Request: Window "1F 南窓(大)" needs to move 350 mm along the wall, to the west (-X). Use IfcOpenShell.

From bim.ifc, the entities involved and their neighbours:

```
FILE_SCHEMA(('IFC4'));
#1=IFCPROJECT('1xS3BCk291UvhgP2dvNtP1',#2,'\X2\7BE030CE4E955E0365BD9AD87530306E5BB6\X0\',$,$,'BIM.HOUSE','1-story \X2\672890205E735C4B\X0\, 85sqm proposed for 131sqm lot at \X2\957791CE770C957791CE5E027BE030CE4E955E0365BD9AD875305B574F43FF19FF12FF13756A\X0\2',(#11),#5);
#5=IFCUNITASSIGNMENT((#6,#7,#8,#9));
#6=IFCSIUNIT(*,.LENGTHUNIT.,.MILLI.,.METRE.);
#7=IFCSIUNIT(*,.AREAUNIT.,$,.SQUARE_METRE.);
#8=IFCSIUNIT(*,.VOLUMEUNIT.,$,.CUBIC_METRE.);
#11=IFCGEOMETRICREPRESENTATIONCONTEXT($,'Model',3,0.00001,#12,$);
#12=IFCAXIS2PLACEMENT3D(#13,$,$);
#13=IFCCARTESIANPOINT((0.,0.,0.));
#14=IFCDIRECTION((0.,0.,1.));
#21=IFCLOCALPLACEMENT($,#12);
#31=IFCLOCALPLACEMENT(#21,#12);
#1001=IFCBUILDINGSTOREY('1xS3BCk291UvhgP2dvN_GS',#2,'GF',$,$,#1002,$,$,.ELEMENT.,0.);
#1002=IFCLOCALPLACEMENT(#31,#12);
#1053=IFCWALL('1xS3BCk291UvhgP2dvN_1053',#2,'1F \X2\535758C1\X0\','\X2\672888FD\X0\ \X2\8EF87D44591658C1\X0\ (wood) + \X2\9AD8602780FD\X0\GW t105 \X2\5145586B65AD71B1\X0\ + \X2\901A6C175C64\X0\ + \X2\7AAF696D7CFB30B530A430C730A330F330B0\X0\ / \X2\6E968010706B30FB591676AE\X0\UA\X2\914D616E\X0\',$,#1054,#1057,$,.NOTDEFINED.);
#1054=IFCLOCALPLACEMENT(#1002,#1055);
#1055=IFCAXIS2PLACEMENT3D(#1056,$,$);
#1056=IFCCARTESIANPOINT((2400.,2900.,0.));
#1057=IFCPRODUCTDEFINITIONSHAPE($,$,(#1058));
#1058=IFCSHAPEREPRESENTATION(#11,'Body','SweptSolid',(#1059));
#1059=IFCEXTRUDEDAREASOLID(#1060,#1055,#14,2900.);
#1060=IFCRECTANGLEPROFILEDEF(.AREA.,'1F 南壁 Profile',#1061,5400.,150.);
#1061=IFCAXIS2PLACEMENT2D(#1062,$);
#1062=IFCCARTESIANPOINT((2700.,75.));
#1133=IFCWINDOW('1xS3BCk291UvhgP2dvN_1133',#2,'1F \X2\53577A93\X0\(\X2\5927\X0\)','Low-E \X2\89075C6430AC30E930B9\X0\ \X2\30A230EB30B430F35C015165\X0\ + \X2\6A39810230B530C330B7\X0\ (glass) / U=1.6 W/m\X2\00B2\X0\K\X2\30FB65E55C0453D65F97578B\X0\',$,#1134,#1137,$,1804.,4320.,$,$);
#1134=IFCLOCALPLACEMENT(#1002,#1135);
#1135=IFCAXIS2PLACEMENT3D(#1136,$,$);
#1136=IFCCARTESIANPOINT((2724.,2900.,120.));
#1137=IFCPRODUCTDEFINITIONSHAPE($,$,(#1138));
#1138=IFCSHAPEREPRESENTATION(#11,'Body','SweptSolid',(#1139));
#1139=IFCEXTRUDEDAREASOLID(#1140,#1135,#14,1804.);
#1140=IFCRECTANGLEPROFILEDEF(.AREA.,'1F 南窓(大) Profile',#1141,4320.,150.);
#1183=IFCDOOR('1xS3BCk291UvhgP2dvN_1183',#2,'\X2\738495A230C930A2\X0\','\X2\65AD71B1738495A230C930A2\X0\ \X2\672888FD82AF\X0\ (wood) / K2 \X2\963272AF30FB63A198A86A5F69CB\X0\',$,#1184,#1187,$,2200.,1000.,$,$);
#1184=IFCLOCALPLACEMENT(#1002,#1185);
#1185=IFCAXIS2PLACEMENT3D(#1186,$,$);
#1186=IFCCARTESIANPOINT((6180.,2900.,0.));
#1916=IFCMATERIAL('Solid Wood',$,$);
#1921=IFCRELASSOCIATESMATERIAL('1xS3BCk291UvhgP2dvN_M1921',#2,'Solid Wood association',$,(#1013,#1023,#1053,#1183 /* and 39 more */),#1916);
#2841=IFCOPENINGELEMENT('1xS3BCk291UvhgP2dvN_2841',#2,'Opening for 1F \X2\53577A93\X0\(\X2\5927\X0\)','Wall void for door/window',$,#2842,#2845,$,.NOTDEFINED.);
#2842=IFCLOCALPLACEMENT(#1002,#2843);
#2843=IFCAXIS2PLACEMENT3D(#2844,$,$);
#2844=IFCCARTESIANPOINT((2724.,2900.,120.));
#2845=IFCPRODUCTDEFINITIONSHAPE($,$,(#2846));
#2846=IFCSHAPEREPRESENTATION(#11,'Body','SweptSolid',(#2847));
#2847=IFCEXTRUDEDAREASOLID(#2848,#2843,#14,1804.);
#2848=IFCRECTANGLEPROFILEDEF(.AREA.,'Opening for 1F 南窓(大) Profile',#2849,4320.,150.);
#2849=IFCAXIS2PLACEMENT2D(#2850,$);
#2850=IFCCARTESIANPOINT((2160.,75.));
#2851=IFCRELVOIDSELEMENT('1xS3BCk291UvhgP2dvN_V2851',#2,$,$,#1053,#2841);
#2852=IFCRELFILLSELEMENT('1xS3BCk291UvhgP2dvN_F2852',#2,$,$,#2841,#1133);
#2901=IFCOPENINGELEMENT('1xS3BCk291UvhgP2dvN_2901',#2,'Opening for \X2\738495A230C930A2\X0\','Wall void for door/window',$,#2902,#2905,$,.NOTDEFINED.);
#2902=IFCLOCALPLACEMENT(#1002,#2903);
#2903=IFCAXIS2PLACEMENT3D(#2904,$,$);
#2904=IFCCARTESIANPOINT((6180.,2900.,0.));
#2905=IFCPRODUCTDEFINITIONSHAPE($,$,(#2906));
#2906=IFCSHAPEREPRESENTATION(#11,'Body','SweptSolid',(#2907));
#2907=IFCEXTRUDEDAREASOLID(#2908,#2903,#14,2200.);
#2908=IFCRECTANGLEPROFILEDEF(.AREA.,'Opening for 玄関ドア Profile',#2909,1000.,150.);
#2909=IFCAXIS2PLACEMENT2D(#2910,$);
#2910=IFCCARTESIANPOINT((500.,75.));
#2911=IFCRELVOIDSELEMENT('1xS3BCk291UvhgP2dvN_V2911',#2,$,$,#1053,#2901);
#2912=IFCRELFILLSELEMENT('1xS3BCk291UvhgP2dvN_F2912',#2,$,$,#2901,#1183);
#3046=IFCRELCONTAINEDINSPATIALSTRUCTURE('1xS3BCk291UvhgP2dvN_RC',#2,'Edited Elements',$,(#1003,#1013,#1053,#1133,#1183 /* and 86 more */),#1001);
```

```python
import ifcopenshell
import ifcopenshell.api.geometry
import ifcopenshell.util.placement

model = ifcopenshell.open("bim.ifc")

window = model.by_guid("1xS3BCk291UvhgP2dvN_1133")
opening = window.FillsVoids[0].RelatingOpeningElement
wall = opening.VoidsElements[0].RelatingBuildingElement

wall_matrix = ifcopenshell.util.placement.get_local_placement(wall.ObjectPlacement)
shift = wall_matrix[:3, 0] * -350.0
before = ifcopenshell.util.placement.get_local_placement(window.ObjectPlacement)[:3, 3].copy()

# The window is not placed relative to its opening, so move both.
for product in (opening, window):
    matrix = ifcopenshell.util.placement.get_local_placement(product.ObjectPlacement)
    matrix[:3, 3] += shift
    ifcopenshell.api.geometry.edit_object_placement(model, product=product, matrix=matrix, is_si=False)

after = ifcopenshell.util.placement.get_local_placement(window.ObjectPlacement)[:3, 3]
print("window moved by", (after - before).round(3) + 0.0)

model.write("bim-out.ifc")
```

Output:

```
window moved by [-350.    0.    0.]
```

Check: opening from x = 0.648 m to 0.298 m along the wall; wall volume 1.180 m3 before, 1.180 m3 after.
